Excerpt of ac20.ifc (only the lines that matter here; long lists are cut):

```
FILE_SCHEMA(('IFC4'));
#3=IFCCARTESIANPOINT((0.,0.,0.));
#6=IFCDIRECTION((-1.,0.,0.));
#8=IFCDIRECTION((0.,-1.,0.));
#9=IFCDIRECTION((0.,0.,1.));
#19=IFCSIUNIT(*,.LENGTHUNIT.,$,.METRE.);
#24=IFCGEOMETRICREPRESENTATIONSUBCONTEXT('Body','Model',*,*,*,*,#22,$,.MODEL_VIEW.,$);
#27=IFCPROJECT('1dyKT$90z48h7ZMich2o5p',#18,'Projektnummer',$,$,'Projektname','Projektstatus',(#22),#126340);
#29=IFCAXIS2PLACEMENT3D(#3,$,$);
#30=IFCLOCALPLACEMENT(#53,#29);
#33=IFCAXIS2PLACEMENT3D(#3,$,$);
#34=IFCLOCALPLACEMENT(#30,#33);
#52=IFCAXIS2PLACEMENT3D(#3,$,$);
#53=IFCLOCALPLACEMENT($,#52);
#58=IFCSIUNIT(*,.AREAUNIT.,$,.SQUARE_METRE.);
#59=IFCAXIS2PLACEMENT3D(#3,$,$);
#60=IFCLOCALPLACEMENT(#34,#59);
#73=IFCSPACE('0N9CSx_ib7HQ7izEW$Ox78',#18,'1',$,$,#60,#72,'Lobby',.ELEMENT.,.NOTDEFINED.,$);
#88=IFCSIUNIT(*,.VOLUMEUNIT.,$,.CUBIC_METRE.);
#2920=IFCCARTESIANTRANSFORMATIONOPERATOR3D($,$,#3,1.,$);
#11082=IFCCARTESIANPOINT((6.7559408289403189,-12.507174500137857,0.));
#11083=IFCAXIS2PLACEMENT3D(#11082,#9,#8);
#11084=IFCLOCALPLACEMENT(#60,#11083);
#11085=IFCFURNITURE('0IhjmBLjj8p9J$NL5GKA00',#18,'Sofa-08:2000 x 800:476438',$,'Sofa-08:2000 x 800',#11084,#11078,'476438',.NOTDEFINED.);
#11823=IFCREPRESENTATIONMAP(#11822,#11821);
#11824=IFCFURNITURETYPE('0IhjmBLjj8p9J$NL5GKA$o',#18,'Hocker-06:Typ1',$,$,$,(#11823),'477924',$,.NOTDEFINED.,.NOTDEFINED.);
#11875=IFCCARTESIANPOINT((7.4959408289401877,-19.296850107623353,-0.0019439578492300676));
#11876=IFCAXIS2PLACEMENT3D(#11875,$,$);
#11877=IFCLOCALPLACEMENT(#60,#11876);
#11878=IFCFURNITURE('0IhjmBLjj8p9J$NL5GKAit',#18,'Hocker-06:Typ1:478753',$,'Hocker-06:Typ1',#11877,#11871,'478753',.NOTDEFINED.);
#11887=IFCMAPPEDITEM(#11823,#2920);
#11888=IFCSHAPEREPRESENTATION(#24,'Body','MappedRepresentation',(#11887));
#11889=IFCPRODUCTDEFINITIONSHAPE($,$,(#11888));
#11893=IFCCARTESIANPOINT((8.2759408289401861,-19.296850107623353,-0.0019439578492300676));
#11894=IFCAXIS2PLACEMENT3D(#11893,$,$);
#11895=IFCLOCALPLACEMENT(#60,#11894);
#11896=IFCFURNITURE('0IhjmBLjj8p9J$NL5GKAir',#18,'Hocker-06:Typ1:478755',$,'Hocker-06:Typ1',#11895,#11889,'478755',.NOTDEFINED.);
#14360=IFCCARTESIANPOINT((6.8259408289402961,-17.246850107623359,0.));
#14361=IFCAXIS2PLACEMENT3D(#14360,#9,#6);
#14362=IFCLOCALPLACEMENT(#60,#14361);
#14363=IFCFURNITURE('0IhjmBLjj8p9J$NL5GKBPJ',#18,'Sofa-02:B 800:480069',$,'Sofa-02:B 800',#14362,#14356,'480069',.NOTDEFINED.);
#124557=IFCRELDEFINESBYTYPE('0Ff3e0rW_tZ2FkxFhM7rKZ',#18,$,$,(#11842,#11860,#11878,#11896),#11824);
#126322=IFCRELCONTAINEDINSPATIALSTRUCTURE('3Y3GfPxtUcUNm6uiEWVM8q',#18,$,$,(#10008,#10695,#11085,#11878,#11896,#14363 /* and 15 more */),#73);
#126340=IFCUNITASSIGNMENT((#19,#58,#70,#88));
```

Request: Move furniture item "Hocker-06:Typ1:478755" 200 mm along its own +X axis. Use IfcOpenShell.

```python
import ifcopenshell
import ifcopenshell.api.geometry
import ifcopenshell.util.placement

model = ifcopenshell.open("ac20.ifc")

item = model.by_guid("0IhjmBLjj8p9J$NL5GKAir")
matrix = ifcopenshell.util.placement.get_local_placement(item.ObjectPlacement)
matrix[:3, 3] += matrix[:3, 0] * 0.2
ifcopenshell.api.geometry.edit_object_placement(model, product=item, matrix=matrix, is_si=False)

print(ifcopenshell.util.placement.get_local_placement(item.ObjectPlacement).round(3) + 0.0)

model.write("ac20_v2.ifc")
```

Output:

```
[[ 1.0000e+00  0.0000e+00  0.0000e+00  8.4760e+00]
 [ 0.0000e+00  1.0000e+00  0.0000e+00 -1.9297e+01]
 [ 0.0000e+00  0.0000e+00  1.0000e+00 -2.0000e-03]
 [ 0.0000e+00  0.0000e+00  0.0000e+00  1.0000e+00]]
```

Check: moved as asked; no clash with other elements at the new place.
